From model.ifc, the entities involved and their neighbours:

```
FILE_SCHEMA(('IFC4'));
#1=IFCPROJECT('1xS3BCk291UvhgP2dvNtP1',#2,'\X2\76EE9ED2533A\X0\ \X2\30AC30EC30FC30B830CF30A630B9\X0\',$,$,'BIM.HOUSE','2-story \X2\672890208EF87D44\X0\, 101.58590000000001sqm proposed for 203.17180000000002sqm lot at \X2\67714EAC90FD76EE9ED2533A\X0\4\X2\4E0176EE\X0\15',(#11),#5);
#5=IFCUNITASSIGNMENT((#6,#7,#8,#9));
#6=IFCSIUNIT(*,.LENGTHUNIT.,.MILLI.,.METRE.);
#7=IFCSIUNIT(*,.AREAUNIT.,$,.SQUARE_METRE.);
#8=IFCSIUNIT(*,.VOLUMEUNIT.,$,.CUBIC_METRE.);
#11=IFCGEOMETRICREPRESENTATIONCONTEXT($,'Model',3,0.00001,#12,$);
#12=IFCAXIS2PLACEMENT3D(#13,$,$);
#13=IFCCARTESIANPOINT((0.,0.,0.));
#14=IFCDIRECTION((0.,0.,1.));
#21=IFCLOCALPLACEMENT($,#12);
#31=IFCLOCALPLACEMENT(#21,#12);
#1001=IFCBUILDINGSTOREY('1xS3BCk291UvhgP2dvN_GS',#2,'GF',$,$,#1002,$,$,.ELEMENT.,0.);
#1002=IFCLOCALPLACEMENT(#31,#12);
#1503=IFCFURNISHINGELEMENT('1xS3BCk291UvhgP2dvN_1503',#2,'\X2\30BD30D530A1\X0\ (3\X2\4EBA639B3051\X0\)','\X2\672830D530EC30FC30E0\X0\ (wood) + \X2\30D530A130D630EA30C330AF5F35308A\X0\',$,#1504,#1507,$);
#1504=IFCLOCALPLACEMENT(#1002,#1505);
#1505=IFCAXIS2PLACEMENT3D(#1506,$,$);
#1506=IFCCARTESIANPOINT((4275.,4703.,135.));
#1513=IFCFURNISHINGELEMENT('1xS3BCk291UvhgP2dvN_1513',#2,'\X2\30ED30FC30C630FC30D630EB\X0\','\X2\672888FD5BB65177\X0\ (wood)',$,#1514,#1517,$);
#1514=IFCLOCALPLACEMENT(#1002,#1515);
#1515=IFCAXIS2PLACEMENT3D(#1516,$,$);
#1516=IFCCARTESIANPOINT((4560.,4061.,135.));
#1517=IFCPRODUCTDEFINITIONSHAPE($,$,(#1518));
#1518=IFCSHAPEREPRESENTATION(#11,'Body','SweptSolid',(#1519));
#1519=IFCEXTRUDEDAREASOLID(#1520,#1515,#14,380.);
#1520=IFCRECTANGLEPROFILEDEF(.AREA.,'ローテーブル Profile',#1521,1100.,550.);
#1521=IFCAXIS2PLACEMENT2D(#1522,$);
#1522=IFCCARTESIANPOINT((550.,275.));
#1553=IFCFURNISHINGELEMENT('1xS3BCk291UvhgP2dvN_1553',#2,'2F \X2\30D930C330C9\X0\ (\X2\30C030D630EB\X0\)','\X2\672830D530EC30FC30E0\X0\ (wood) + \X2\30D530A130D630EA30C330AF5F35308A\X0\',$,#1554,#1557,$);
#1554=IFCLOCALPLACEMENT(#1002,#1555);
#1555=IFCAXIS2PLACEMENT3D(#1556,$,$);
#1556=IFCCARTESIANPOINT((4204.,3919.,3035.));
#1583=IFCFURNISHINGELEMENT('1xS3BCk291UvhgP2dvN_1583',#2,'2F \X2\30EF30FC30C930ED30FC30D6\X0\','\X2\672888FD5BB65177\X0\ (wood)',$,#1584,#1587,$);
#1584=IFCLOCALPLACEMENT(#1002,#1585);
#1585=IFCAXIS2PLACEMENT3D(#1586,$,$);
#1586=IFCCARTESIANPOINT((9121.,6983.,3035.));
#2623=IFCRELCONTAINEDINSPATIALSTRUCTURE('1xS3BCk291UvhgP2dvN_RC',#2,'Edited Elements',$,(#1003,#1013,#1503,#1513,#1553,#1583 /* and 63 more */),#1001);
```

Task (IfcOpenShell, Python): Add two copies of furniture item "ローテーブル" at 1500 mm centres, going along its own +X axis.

```python
import ifcopenshell
import ifcopenshell.api.geometry
import ifcopenshell.api.root
import ifcopenshell.util.element
import ifcopenshell.util.placement
import ifcopenshell.util.unit

model = ifcopenshell.open("model.ifc")
unit_scale = ifcopenshell.util.unit.calculate_unit_scale(model)


def reuse_history(source, copy):
    """copy_class also copies each property set's owner history, people and application; keep the originals."""
    for rel in copy.IsDefinedBy:
        if rel.is_a("IfcRelDefinesByProperties") and (history := rel.RelatingPropertyDefinition.OwnerHistory):
            rel.RelatingPropertyDefinition.OwnerHistory = source.OwnerHistory
            ifcopenshell.util.element.remove_deep2(model, history)


source = model.by_guid("1xS3BCk291UvhgP2dvN_1513")
base = ifcopenshell.util.placement.get_local_placement(source.ObjectPlacement)
step = base[:3, 0] * 1.5 / unit_scale

for i in range(1, 3):
    copy = ifcopenshell.api.root.copy_class(model, product=source)
    copy.Representation = ifcopenshell.util.element.copy_deep(
        model, source.Representation, exclude=["IfcGeometricRepresentationContext", "IfcRepresentationMap"]
    )
    reuse_history(source, copy)
    matrix = base.copy()
    matrix[:3, 3] += i * step
    print("added at", matrix[:3, 3].round(3) + 0.0)
    ifcopenshell.api.geometry.edit_object_placement(model, product=copy, matrix=matrix, is_si=False)

model.write("model_edited.ifc")
```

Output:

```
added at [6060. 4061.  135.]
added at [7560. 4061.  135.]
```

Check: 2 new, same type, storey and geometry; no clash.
